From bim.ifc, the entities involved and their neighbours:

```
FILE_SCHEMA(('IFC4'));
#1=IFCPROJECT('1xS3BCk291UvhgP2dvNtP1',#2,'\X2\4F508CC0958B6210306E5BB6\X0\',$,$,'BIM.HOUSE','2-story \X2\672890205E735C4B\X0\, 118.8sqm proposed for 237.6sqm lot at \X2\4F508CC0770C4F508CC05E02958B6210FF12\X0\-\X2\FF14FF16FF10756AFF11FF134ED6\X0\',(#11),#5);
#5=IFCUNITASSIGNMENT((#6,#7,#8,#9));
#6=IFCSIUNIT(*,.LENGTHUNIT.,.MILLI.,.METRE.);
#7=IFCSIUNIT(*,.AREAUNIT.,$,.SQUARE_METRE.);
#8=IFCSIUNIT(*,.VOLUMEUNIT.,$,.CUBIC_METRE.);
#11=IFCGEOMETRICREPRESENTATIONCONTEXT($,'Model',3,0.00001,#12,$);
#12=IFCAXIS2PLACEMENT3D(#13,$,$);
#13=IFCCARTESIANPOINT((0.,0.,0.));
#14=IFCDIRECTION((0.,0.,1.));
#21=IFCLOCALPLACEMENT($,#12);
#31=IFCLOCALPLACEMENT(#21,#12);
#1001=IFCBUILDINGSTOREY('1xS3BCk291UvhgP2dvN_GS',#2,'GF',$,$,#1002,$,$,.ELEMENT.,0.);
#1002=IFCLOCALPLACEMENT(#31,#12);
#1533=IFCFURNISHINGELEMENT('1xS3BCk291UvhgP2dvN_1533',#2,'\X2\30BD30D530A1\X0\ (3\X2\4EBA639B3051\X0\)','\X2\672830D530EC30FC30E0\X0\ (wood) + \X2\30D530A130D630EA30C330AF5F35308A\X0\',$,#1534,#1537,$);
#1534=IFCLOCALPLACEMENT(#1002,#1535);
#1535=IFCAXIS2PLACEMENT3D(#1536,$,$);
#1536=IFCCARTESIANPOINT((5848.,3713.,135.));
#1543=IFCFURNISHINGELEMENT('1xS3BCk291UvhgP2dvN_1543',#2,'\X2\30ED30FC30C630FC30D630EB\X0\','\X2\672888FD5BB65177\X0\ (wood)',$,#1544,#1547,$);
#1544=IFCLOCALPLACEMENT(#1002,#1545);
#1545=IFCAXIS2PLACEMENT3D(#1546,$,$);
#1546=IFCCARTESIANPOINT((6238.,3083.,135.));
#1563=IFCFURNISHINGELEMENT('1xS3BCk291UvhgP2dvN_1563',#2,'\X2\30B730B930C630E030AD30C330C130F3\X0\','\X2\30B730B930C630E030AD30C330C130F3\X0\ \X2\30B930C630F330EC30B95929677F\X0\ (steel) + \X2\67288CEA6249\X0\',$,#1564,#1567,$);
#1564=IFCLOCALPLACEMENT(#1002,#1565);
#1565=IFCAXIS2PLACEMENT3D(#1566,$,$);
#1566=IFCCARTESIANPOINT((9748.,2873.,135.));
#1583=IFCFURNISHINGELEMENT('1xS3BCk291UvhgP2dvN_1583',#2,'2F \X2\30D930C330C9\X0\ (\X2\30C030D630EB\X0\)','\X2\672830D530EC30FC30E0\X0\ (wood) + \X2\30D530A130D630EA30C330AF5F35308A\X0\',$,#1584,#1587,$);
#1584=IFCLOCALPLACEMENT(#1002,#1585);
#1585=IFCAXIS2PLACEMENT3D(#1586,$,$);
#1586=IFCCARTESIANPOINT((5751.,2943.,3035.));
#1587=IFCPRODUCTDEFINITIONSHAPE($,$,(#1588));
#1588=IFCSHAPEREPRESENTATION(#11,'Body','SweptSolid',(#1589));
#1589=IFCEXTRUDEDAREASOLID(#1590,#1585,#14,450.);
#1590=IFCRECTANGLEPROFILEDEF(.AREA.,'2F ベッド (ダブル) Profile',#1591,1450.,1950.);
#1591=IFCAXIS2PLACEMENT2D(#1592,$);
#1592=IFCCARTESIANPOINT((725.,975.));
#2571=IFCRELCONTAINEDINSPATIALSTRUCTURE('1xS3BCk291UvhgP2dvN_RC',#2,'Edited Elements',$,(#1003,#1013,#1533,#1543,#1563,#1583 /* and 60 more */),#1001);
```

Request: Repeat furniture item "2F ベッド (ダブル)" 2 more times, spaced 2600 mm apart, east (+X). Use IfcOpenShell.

```python
import numpy as np
import ifcopenshell
import ifcopenshell.api.geometry
import ifcopenshell.api.root
import ifcopenshell.util.element
import ifcopenshell.util.placement
import ifcopenshell.util.unit

model = ifcopenshell.open("bim.ifc")
unit_scale = ifcopenshell.util.unit.calculate_unit_scale(model)


def reuse_history(source, copy):
    """copy_class also copies each property set's owner history, people and application; keep the originals."""
    for rel in copy.IsDefinedBy:
        if rel.is_a("IfcRelDefinesByProperties") and (history := rel.RelatingPropertyDefinition.OwnerHistory):
            rel.RelatingPropertyDefinition.OwnerHistory = source.OwnerHistory
            ifcopenshell.util.element.remove_deep2(model, history)


source = model.by_guid("1xS3BCk291UvhgP2dvN_1583")
base = ifcopenshell.util.placement.get_local_placement(source.ObjectPlacement)
step = np.array([1.0, 0.0, 0.0]) * 2.6 / unit_scale

for i in range(1, 3):
    copy = ifcopenshell.api.root.copy_class(model, product=source)
    copy.Representation = ifcopenshell.util.element.copy_deep(
        model, source.Representation, exclude=["IfcGeometricRepresentationContext", "IfcRepresentationMap"]
    )
    reuse_history(source, copy)
    matrix = base.copy()
    matrix[:3, 3] += i * step
    print("added at", matrix[:3, 3].round(3) + 0.0)
    ifcopenshell.api.geometry.edit_object_placement(model, product=copy, matrix=matrix, is_si=False)

model.write("bim-out.ifc")
```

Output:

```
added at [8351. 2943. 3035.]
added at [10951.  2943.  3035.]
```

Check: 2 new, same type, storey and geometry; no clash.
